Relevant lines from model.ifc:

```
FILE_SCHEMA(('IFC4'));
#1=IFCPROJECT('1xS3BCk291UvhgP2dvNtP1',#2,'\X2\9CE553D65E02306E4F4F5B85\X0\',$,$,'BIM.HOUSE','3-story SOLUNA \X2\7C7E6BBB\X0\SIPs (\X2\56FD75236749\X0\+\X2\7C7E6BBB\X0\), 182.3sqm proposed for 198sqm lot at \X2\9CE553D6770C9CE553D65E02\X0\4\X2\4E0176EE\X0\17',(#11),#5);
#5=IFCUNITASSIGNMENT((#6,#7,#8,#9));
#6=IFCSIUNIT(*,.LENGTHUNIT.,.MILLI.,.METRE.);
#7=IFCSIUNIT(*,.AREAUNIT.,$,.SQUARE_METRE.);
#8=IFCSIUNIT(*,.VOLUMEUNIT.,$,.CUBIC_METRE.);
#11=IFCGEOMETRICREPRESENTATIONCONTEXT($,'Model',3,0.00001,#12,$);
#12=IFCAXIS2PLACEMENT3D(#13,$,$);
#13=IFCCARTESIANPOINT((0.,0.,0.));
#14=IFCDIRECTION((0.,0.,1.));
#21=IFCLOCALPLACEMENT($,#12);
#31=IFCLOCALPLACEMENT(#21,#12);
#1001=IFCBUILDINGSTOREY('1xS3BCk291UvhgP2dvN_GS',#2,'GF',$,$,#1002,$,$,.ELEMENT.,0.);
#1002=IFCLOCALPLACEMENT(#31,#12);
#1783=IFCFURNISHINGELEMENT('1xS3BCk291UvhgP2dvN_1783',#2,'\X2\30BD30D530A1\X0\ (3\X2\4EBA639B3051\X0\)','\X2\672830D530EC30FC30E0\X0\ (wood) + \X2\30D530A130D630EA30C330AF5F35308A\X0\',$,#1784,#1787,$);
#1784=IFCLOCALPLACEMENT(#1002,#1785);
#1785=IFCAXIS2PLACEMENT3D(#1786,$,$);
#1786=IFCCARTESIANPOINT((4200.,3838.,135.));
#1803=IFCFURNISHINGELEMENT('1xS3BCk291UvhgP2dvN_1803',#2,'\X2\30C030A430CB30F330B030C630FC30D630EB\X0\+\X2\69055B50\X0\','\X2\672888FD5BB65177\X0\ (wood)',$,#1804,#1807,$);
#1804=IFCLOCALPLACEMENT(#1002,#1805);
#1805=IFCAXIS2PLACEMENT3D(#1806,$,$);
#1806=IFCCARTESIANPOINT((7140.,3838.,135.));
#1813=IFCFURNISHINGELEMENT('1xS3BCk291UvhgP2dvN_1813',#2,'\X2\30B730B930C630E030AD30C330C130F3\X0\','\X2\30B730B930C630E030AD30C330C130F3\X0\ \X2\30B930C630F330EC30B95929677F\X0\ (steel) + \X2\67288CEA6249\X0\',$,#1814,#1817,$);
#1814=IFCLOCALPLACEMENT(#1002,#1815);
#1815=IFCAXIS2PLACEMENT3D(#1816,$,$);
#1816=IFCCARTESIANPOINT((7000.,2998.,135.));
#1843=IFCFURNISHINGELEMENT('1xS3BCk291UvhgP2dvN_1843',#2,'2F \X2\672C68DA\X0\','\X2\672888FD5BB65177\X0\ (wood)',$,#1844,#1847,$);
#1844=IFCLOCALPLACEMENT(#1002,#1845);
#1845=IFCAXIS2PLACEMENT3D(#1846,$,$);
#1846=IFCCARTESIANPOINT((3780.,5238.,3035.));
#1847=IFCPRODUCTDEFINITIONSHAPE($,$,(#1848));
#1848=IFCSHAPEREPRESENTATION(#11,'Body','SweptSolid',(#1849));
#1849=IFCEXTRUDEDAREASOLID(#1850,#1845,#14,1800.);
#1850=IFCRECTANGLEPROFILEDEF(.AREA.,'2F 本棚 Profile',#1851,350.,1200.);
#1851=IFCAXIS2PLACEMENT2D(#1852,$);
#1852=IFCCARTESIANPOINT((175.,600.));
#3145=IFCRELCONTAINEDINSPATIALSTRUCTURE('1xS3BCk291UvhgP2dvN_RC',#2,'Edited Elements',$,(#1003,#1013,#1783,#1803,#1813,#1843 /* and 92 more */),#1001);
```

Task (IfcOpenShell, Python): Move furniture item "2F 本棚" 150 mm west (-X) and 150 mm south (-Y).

```python
import ifcopenshell
import ifcopenshell.api.geometry
import ifcopenshell.util.placement

model = ifcopenshell.open("model.ifc")

item = model.by_guid("1xS3BCk291UvhgP2dvN_1843")
matrix = ifcopenshell.util.placement.get_local_placement(item.ObjectPlacement)
matrix[0, 3] -= 150.0
matrix[1, 3] -= 150.0
ifcopenshell.api.geometry.edit_object_placement(model, product=item, matrix=matrix, is_si=False)

print(ifcopenshell.util.placement.get_local_placement(item.ObjectPlacement).round(3) + 0.0)

model.write("model_updated.ifc")
```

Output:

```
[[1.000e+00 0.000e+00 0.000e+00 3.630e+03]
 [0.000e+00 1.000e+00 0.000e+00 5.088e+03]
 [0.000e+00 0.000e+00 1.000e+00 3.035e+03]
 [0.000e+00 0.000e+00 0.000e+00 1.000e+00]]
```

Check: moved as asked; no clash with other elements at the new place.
